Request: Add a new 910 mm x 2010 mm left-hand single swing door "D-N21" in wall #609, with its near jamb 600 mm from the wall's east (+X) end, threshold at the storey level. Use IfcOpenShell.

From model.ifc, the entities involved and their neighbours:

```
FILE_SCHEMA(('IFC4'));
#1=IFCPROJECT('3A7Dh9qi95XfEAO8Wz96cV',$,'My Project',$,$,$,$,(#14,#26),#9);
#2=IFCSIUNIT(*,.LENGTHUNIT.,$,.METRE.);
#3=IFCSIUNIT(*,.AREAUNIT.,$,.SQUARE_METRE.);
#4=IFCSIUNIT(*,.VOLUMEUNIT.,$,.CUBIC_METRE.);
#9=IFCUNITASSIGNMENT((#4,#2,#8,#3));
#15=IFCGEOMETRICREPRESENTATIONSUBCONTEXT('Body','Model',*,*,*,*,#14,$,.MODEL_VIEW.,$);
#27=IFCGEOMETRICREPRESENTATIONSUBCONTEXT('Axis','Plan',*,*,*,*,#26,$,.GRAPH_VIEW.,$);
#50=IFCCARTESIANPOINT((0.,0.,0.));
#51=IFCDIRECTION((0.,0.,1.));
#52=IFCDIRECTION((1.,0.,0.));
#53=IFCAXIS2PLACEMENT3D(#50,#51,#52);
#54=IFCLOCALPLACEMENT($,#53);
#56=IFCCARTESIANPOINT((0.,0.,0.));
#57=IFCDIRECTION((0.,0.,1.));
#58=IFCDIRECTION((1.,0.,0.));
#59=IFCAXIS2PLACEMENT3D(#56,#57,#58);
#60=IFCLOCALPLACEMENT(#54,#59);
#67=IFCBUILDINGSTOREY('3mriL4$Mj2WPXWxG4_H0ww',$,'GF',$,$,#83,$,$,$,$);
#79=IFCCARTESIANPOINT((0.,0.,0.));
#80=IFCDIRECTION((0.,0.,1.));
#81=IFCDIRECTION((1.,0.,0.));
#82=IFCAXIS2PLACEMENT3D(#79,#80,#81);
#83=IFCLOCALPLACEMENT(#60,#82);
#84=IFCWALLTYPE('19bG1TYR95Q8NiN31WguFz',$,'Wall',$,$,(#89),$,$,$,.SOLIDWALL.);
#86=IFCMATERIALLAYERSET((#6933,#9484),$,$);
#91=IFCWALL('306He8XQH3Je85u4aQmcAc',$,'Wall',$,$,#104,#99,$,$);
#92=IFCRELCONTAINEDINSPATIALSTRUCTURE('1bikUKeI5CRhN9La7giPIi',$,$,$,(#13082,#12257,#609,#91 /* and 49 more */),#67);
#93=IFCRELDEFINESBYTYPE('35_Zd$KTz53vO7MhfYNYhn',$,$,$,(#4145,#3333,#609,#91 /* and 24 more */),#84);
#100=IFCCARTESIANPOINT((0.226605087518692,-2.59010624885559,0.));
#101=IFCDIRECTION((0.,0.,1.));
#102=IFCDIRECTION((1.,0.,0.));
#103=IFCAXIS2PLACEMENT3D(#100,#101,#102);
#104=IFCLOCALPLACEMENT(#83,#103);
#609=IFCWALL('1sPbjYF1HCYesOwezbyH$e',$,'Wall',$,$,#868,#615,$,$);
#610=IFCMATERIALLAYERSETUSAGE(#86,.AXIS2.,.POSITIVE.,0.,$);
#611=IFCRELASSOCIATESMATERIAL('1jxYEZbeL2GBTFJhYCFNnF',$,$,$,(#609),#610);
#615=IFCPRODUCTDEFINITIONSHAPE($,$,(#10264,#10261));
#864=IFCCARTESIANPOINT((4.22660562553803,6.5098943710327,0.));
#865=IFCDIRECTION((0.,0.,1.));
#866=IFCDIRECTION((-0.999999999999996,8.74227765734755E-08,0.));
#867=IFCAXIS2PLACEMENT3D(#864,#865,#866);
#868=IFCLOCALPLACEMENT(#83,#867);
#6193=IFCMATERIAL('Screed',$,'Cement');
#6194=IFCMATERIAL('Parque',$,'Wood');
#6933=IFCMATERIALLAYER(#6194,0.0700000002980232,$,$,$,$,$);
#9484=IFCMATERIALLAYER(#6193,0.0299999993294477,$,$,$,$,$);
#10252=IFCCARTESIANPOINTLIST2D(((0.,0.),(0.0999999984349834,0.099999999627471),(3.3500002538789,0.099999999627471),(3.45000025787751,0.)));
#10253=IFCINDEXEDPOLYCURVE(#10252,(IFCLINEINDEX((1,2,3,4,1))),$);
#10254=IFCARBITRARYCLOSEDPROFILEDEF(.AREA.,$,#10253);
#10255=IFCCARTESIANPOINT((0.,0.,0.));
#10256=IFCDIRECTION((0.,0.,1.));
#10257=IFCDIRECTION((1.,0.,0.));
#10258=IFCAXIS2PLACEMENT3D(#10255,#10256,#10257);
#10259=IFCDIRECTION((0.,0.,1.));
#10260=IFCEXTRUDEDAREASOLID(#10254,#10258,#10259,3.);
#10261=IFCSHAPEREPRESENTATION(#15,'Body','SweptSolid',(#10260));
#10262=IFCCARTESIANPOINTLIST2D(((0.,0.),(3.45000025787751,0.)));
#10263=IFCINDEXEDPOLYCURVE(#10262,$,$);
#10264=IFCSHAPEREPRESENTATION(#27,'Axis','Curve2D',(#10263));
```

```python
import numpy as np
import ifcopenshell
import ifcopenshell.api.feature
import ifcopenshell.api.geometry
import ifcopenshell.api.root
import ifcopenshell.api.spatial
import ifcopenshell.geom
import ifcopenshell.util.element
import ifcopenshell.util.placement
import ifcopenshell.util.representation
import ifcopenshell.util.shape
import ifcopenshell.util.unit

model = ifcopenshell.open("model.ifc")
unit_scale = ifcopenshell.util.unit.calculate_unit_scale(model)
settings = ifcopenshell.geom.settings()


def volume(element):
    """Net volume in cubic metres, openings subtracted."""
    shape = ifcopenshell.geom.create_shape(settings, element)
    return ifcopenshell.util.shape.get_volume(shape.geometry)


wall = model.by_id(609)
storey = ifcopenshell.util.element.get_container(wall, ifc_class="IfcBuildingStorey")
context = ifcopenshell.util.representation.get_context(model, "Model", "Body", "MODEL_VIEW")
before = volume(wall)

width, height, from_end, sill = 0.91, 2.01, 0.6, 0.0  # metres

# The wall runs along its own X axis, and the end named is its -X end.
wall_shape = ifcopenshell.geom.create_shape(settings, wall)
x, y, z = ifcopenshell.util.shape.get_vertices(wall_shape.geometry).T
start = x.min() + from_end
face, thickness = float(y.min()), float(y.max() - y.min())
wall_matrix = ifcopenshell.util.placement.get_local_placement(wall.ObjectPlacement)
level = ifcopenshell.util.placement.get_local_placement(storey.ObjectPlacement)[2, 3]


def in_wall(x, y):
    """Placement at x, y metres in the wall's axes, at sill height."""
    matrix = wall_matrix.copy()
    matrix[:, 3] = wall_matrix @ np.array([x / unit_scale, y / unit_scale, 0.0, 1.0])
    matrix[2, 3] = level + sill / unit_scale
    return matrix


# Opening: a box that overshoots both wall faces by 50 mm.
opening = ifcopenshell.api.root.create_entity(model, ifc_class="IfcOpeningElement", predefined_type="OPENING")
box = ifcopenshell.api.geometry.add_wall_representation(
    model, context=context, length=width, height=height, thickness=thickness + 0.1
)
ifcopenshell.api.geometry.assign_representation(model, product=opening, representation=box)
ifcopenshell.api.geometry.edit_object_placement(model, product=opening, matrix=in_wall(start, face - 0.05), is_si=False)
ifcopenshell.api.feature.add_feature(model, feature=opening, element=wall)

door = ifcopenshell.api.root.create_entity(model, ifc_class="IfcDoor", name="D-N21", predefined_type="DOOR")
door.OverallWidth, door.OverallHeight = width / unit_scale, height / unit_scale
door.OperationType = "SINGLE_SWING_LEFT"
body = ifcopenshell.api.geometry.add_door_representation(
    model,
    context=context,
    overall_width=door.OverallWidth,
    overall_height=door.OverallHeight,
    operation_type="SINGLE_SWING_LEFT",
    lining_properties={"LiningDepth": thickness / unit_scale, "ThresholdDepth": thickness / unit_scale},
)
ifcopenshell.api.geometry.assign_representation(model, product=door, representation=body)
ifcopenshell.api.spatial.assign_container(model, products=[door], relating_structure=storey)
ifcopenshell.api.feature.add_filling(model, opening=opening, element=door)

# The lining spans the wall, so the door starts at the wall face.
ifcopenshell.api.geometry.edit_object_placement(model, product=door, matrix=in_wall(start, face), is_si=False)

after = volume(wall)

print(f"wall volume {before:.3f} -> {after:.3f} m3")

model.write("model_edited.ifc")
```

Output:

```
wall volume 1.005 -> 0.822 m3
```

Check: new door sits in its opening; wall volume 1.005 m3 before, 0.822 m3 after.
